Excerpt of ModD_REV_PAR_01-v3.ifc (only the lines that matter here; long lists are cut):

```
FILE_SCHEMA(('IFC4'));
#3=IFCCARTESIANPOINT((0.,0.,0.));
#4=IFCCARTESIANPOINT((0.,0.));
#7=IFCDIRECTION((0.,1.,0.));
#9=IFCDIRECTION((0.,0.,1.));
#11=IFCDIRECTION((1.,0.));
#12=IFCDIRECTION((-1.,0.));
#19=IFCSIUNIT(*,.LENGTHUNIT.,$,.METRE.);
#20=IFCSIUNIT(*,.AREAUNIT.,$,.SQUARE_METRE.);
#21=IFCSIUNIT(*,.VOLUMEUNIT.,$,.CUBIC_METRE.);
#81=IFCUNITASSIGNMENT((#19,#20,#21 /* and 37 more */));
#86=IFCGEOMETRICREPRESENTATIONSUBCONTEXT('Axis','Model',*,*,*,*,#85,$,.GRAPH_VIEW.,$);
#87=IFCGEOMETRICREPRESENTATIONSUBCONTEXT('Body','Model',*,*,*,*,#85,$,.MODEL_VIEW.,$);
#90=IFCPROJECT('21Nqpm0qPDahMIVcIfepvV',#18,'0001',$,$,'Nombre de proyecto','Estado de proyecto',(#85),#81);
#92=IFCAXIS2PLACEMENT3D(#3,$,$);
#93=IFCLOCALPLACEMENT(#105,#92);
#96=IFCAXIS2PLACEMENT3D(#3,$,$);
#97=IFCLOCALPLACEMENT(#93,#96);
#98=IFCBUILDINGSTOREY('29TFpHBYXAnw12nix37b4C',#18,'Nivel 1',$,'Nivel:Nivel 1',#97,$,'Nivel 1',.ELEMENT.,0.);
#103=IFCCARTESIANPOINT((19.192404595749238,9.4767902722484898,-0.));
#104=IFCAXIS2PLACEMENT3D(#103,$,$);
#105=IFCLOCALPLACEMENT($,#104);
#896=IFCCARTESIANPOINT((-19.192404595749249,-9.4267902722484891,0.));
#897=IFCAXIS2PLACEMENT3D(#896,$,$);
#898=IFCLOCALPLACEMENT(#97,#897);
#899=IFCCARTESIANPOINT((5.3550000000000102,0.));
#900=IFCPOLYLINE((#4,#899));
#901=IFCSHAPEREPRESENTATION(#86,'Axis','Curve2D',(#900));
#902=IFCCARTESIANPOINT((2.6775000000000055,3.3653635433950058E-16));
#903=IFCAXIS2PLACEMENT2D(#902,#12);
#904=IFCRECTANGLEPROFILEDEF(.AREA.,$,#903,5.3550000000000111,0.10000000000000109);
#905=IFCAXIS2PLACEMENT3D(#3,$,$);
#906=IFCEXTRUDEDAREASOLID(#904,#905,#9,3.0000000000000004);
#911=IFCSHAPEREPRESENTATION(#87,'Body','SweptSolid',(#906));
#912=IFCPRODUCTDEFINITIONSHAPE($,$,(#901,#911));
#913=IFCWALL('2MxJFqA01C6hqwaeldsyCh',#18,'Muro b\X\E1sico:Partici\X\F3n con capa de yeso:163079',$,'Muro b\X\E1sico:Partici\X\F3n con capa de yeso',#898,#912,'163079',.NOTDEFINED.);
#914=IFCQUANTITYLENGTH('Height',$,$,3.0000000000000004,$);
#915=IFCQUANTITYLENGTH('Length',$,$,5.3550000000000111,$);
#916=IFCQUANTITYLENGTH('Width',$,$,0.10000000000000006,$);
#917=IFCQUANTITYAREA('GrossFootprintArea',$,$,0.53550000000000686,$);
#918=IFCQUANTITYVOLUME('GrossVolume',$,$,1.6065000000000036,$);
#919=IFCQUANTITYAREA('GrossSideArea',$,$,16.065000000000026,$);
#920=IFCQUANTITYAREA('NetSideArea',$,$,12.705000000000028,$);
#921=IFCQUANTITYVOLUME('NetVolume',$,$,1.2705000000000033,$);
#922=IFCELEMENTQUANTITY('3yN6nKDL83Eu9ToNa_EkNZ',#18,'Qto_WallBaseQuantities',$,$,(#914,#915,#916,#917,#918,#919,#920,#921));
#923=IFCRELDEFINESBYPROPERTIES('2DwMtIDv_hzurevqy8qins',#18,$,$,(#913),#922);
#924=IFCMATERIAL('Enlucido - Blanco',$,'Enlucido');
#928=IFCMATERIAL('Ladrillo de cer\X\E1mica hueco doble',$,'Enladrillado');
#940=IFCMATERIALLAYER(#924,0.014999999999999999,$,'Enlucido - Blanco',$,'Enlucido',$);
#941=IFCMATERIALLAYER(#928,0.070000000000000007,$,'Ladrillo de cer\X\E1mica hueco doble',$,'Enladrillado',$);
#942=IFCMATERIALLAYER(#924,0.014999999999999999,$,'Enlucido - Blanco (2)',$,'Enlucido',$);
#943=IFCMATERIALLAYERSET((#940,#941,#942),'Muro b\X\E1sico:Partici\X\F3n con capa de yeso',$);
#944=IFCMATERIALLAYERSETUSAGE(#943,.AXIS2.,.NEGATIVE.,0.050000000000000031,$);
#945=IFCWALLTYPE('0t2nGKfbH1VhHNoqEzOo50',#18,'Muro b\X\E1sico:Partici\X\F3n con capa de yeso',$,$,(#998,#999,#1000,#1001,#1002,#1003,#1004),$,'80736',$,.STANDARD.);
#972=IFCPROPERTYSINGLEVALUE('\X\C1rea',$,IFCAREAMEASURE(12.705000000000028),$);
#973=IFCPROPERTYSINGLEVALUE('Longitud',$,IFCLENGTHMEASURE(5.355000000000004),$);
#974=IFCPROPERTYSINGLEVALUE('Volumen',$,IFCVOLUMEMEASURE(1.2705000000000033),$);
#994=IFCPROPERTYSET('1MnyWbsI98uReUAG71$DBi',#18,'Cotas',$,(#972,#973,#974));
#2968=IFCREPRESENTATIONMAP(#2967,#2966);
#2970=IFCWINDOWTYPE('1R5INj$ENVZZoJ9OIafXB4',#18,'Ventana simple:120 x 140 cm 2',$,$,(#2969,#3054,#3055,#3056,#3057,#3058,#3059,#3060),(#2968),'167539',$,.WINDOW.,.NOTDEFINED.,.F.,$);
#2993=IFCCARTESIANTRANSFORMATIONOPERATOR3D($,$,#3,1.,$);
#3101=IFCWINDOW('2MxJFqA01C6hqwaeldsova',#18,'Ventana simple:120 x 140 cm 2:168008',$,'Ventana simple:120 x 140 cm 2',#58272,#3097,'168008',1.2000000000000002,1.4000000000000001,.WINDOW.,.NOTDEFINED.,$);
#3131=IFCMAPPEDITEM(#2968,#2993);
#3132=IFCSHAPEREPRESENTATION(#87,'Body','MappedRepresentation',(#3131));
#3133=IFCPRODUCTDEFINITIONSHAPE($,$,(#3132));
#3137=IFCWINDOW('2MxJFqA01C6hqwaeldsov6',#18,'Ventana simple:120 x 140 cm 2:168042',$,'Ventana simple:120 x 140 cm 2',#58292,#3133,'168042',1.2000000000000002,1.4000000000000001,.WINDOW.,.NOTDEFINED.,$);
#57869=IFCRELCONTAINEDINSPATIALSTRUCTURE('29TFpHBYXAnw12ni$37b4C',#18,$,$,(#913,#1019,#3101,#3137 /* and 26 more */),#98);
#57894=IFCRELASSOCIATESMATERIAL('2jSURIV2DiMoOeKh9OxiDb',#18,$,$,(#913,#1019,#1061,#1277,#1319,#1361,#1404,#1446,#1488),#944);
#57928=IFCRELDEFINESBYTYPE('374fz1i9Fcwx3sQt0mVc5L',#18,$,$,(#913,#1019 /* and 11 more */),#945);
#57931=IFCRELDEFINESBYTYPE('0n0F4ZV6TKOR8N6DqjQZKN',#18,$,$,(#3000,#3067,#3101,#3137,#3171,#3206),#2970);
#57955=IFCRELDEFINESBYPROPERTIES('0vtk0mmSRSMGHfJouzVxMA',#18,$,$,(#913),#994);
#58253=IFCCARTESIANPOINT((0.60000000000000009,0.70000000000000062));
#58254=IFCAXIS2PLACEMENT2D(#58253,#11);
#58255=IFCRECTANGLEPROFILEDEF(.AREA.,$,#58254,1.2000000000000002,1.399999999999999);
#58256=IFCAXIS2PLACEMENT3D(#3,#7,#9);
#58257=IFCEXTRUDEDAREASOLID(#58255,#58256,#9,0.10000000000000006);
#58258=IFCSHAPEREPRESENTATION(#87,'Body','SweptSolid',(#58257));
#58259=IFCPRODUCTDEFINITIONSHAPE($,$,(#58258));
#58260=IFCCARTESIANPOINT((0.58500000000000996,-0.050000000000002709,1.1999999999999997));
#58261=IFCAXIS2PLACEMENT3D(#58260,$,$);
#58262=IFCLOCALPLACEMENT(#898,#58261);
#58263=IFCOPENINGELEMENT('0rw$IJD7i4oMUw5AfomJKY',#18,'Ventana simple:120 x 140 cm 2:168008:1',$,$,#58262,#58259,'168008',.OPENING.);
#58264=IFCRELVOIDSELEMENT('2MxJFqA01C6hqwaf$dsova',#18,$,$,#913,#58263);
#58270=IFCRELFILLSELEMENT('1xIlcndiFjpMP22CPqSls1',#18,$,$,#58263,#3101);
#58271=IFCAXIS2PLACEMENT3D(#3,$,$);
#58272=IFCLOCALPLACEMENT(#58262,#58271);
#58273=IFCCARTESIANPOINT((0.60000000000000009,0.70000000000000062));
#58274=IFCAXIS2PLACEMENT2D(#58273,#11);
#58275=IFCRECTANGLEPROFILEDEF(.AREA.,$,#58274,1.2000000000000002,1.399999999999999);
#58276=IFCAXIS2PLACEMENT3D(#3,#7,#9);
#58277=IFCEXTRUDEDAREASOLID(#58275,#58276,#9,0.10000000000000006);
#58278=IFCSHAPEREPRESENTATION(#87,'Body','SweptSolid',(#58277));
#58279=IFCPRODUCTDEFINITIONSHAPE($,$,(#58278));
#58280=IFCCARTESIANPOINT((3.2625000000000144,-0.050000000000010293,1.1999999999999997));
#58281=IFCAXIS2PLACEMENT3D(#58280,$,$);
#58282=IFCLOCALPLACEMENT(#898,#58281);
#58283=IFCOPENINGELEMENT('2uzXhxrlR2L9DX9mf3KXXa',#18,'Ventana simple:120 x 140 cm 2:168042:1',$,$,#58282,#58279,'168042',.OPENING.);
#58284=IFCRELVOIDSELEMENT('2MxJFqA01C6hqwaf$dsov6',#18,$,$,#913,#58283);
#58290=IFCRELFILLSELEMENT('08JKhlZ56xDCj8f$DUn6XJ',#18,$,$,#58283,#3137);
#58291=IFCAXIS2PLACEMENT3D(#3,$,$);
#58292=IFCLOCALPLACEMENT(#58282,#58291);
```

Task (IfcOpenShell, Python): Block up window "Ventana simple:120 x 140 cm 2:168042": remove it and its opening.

```python
import ifcopenshell
import ifcopenshell.api.feature
import ifcopenshell.api.pset
import ifcopenshell.api.root
import ifcopenshell.geom
import ifcopenshell.util.element
import ifcopenshell.util.shape
import ifcopenshell.util.unit

model = ifcopenshell.open("ModD_REV_PAR_01-v3.ifc")
area_scale = ifcopenshell.util.unit.calculate_unit_scale(model, "AREAUNIT")
volume_scale = ifcopenshell.util.unit.calculate_unit_scale(model, "VOLUMEUNIT")
settings = ifcopenshell.geom.settings()


def volume(element):
    """Net volume in cubic metres, openings subtracted."""
    shape = ifcopenshell.geom.create_shape(settings, element)
    return ifcopenshell.util.shape.get_volume(shape.geometry)


window = model.by_guid("2MxJFqA01C6hqwaeldsov6")
opening = window.FillsVoids[0].RelatingOpeningElement
wall = opening.VoidsElements[0].RelatingBuildingElement
before = volume(wall)

ifcopenshell.api.root.remove_product(model, product=window)
ifcopenshell.api.feature.remove_feature(model, feature=opening)

after = volume(wall)
thickness = 0.1  # wall thickness in metres

# Update the wall's stored quantities.
qto = model.by_id(ifcopenshell.util.element.get_pset(wall, "Qto_WallBaseQuantities", should_inherit=False)["id"])
ifcopenshell.api.pset.edit_qto(model, qto=qto, properties={
    "NetSideArea": after / thickness / area_scale,
    "NetVolume": after / volume_scale,
})
pset = model.by_id(ifcopenshell.util.element.get_pset(wall, "Cotas", should_inherit=False)["id"])
ifcopenshell.api.pset.edit_pset(model, pset=pset, properties={
    "Área": model.create_entity("IfcAreaMeasure", after / thickness / area_scale),
    "Volumen": model.create_entity("IfcVolumeMeasure", after / volume_scale),
})

print(f"wall volume {before:.3f} -> {after:.3f} m3")

model.write("ModD_REV_PAR_01-v3_edited.ifc")
```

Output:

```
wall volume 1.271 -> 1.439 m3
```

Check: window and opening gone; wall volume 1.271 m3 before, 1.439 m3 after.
